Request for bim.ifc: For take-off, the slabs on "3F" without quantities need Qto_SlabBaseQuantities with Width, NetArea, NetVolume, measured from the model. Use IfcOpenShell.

First a look at what the model holds.

```python
import ifcopenshell
import ifcopenshell.util.element
import ifcopenshell.util.unit

model = ifcopenshell.open("bim.ifc")
print(model.schema)
for unit_type in ("LENGTHUNIT", "AREAUNIT", "VOLUMEUNIT"):
    print(unit_type, ifcopenshell.util.unit.calculate_unit_scale(model, unit_type))
storey = next(s for s in model.by_type("IfcBuildingStorey") if s.Name == "3F")
slabs = [e for e in ifcopenshell.util.element.get_decomposition(storey) if e.is_a("IfcSlab")]
for e in sorted(slabs, key=lambda e: e.id()):
    print(e.id(), e.is_a(), e.Name, list(ifcopenshell.util.element.get_psets(e, qtos_only=True)), sep=" | ")
```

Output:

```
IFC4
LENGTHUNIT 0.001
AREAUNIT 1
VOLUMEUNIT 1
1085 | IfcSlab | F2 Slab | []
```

```python
import ifcopenshell
import ifcopenshell.api.pset
import ifcopenshell.geom
import ifcopenshell.util.element
import ifcopenshell.util.shape
import ifcopenshell.util.unit

model = ifcopenshell.open("bim.ifc")
unit_scale = ifcopenshell.util.unit.calculate_unit_scale(model)
area_scale = ifcopenshell.util.unit.calculate_unit_scale(model, "AREAUNIT")
volume_scale = ifcopenshell.util.unit.calculate_unit_scale(model, "VOLUMEUNIT")
settings = ifcopenshell.geom.settings()

storey = next(s for s in model.by_type("IfcBuildingStorey") if s.Name == "3F")
slabs = [e for e in ifcopenshell.util.element.get_decomposition(storey) if e.is_a("IfcSlab")]

for e in sorted(slabs, key=lambda e: e.id()):
    if ifcopenshell.util.element.get_psets(e, qtos_only=True, should_inherit=False):
        continue
    # Geometry comes back in metres, in the element's own axes.
    shape = ifcopenshell.geom.create_shape(settings, e)
    values = {
        "Width": ifcopenshell.util.shape.get_z(shape.geometry) / unit_scale,
        "NetArea": ifcopenshell.util.shape.get_footprint_area(shape.geometry) / area_scale,
        "NetVolume": ifcopenshell.util.shape.get_volume(shape.geometry) / volume_scale,
    }
    qto = ifcopenshell.api.pset.add_qto(model, product=e, name="Qto_SlabBaseQuantities")
    ifcopenshell.api.pset.edit_qto(model, qto=qto, properties=values)
    print(e.id(), {k: round(v, 3) for k, v in values.items()})

model.write("bim_edited.ifc")
```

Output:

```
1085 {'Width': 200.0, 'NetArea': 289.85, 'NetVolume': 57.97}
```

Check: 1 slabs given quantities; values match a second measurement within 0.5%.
